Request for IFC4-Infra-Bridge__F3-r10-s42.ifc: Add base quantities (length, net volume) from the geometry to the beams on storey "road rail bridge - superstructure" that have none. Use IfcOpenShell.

First a look at what the model holds.

```python
import ifcopenshell
import ifcopenshell.util.element
import ifcopenshell.util.unit

model = ifcopenshell.open("IFC4-Infra-Bridge__F3-r10-s42.ifc")
print(model.schema)
for unit_type in ("LENGTHUNIT", "AREAUNIT", "VOLUMEUNIT"):
    print(unit_type, ifcopenshell.util.unit.calculate_unit_scale(model, unit_type))
storey = next(s for s in model.by_type("IfcBuildingStorey") if s.Name == "road rail bridge - superstructure")
beams = [e for e in ifcopenshell.util.element.get_decomposition(storey) if e.is_a("IfcBeam")]
for e in sorted(beams, key=lambda e: e.id()):
    print(e.id(), e.is_a(), e.Name, list(ifcopenshell.util.element.get_psets(e, qtos_only=True)), sep=" | ")
```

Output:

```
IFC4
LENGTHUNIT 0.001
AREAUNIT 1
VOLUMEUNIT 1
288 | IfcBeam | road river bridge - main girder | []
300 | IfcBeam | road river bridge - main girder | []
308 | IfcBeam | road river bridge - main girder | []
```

```python
import ifcopenshell
import ifcopenshell.api.pset
import ifcopenshell.geom
import ifcopenshell.util.element
import ifcopenshell.util.shape
import ifcopenshell.util.unit

model = ifcopenshell.open("IFC4-Infra-Bridge__F3-r10-s42.ifc")
unit_scale = ifcopenshell.util.unit.calculate_unit_scale(model)
volume_scale = ifcopenshell.util.unit.calculate_unit_scale(model, "VOLUMEUNIT")
settings = ifcopenshell.geom.settings()

storey = next(s for s in model.by_type("IfcBuildingStorey") if s.Name == "road rail bridge - superstructure")
beams = [e for e in ifcopenshell.util.element.get_decomposition(storey) if e.is_a("IfcBeam")]

for e in sorted(beams, key=lambda e: e.id()):
    if ifcopenshell.util.element.get_psets(e, qtos_only=True, should_inherit=False):
        continue
    # Geometry comes back in metres, in the element's own axes.
    shape = ifcopenshell.geom.create_shape(settings, e)
    values = {
        "Length": ifcopenshell.util.shape.get_max_xyz(shape.geometry) / unit_scale,
        "NetVolume": ifcopenshell.util.shape.get_volume(shape.geometry) / volume_scale,
    }
    qto = ifcopenshell.api.pset.add_qto(model, product=e, name="Qto_BeamBaseQuantities")
    ifcopenshell.api.pset.edit_qto(model, qto=qto, properties=values)
    print(e.id(), {k: round(v, 3) for k, v in values.items()})

model.write("IFC4-Infra-Bridge__F3-r10-s42_edited.ifc")
```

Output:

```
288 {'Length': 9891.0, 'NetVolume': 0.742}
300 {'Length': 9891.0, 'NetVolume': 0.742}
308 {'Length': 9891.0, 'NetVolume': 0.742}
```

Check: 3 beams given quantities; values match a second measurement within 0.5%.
